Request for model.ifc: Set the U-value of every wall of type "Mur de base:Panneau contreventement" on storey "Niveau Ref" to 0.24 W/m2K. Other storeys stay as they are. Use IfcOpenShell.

First a look at what the model holds.

```python
import ifcopenshell
import ifcopenshell.util.element

model = ifcopenshell.open("model.ifc")
print(model.schema)
storey = next(s for s in model.by_type("IfcBuildingStorey") if s.Name == "Niveau Ref")
walls = [e for e in ifcopenshell.util.element.get_decomposition(storey) if e.is_a("IfcWall")]
seen = {}
for e in walls:
    element_type = ifcopenshell.util.element.get_type(e)
    key = (element_type.Name if element_type != e and element_type else None, ifcopenshell.util.element.get_pset(e, "Pset_WallCommon", "ThermalTransmittance"))
    seen[key] = seen.get(key, 0) + 1
for (name, value), count in sorted(seen.items(), key=str):
    print(count, "x", name, "|", value)
```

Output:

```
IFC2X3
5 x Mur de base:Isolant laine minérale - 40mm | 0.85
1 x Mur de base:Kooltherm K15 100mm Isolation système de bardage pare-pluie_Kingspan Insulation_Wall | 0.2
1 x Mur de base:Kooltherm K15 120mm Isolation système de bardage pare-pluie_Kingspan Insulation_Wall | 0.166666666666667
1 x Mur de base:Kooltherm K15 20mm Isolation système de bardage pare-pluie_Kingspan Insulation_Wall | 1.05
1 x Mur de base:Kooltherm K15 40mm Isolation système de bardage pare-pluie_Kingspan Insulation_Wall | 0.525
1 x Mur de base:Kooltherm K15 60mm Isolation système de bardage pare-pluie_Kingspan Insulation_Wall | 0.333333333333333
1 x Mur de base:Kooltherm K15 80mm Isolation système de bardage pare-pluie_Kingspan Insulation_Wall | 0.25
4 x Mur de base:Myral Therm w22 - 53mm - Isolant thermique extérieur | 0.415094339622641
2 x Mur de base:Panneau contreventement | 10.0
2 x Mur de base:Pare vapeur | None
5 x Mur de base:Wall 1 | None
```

```python
import ifcopenshell
import ifcopenshell.api.pset
import ifcopenshell.util.element

model = ifcopenshell.open("model.ifc")

storey = next(s for s in model.by_type("IfcBuildingStorey") if s.Name == "Niveau Ref")
walls = [e for e in ifcopenshell.util.element.get_decomposition(storey) if e.is_a("IfcWall")]

count = 0
for e in walls:
    element_type = ifcopenshell.util.element.get_type(e)
    if element_type in (None, e) or element_type.Name != "Mur de base:Panneau contreventement":
        continue
    # add_pset returns the element's existing set when there is one.
    pset = ifcopenshell.api.pset.add_pset(model, product=e, name="Pset_WallCommon")
    ifcopenshell.api.pset.edit_pset(model, pset=pset, properties={"ThermalTransmittance": 0.24})
    count += 1

print(count, "walls updated")

model.write("model-out.ifc")
```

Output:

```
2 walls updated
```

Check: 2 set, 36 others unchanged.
